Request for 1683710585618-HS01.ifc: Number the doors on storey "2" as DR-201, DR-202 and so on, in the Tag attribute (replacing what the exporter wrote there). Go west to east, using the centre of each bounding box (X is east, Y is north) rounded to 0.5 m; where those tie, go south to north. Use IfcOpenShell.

First a look at what the model holds.

```python
import ifcopenshell
import ifcopenshell.util.element
import ifcopenshell.util.placement

model = ifcopenshell.open("1683710585618-HS01.ifc")
print(model.schema)
storey = next(s for s in model.by_type("IfcBuildingStorey") if s.Name == "2")
doors = [e for e in ifcopenshell.util.element.get_decomposition(storey) if e.is_a("IfcDoor")]
for e in sorted(doors, key=lambda e: e.id()):
    origin = ifcopenshell.util.placement.get_local_placement(e.ObjectPlacement)[:3, 3]
    print(e.id(), e.Tag, e.Name, origin.round(2) + 0.0, sep=" | ")
```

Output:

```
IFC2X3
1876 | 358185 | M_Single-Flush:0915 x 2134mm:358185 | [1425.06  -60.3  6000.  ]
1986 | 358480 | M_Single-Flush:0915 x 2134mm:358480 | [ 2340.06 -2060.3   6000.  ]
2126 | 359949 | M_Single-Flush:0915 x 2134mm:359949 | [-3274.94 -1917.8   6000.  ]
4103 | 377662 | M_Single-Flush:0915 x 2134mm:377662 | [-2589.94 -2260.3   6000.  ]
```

```python
import ifcopenshell
import ifcopenshell.geom
import ifcopenshell.util.element
import ifcopenshell.util.shape

model = ifcopenshell.open("1683710585618-HS01.ifc")
settings = ifcopenshell.geom.settings()
settings.set("use-world-coords", True)


def centre(element):
    shape = ifcopenshell.geom.create_shape(settings, element)
    return ifcopenshell.util.shape.get_bbox_centroid(shape.geometry)


storey = next(s for s in model.by_type("IfcBuildingStorey") if s.Name == "2")
doors = [e for e in ifcopenshell.util.element.get_decomposition(storey) if e.is_a("IfcDoor")]

# Insertion points can sit at a corner or the storey origin, so sort by the geometry (in metres).
centres = {e: centre(e) for e in doors}
doors.sort(key=lambda e: (round(centres[e][0] / 0.5), centres[e][1]))

for i, e in enumerate(doors, start=1):
    number = f"DR-2{i:02d}"
    e.Tag = number
    print(e.id(), number)

model.write("1683710585618-HS01_v2.ifc")
```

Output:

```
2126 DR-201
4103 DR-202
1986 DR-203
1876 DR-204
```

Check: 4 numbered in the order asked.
